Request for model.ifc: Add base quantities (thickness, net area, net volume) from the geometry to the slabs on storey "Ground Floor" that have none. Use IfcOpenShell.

First a look at what the model holds.

```python
import ifcopenshell
import ifcopenshell.util.element
import ifcopenshell.util.unit

model = ifcopenshell.open("model.ifc")
print(model.schema)
for unit_type in ("LENGTHUNIT", "AREAUNIT", "VOLUMEUNIT"):
    print(unit_type, ifcopenshell.util.unit.calculate_unit_scale(model, unit_type))
storey = next(s for s in model.by_type("IfcBuildingStorey") if s.Name == "Ground Floor")
slabs = [e for e in ifcopenshell.util.element.get_decomposition(storey) if e.is_a("IfcSlab")]
for e in sorted(slabs, key=lambda e: e.id()):
    print(e.id(), e.is_a(), e.Name, list(ifcopenshell.util.element.get_psets(e, qtos_only=True)), sep=" | ")
```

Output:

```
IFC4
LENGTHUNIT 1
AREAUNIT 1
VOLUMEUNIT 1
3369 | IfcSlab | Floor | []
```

```python
import ifcopenshell
import ifcopenshell.api.pset
import ifcopenshell.geom
import ifcopenshell.util.element
import ifcopenshell.util.shape
import ifcopenshell.util.unit

model = ifcopenshell.open("model.ifc")
unit_scale = ifcopenshell.util.unit.calculate_unit_scale(model)
area_scale = ifcopenshell.util.unit.calculate_unit_scale(model, "AREAUNIT")
volume_scale = ifcopenshell.util.unit.calculate_unit_scale(model, "VOLUMEUNIT")
settings = ifcopenshell.geom.settings()

storey = next(s for s in model.by_type("IfcBuildingStorey") if s.Name == "Ground Floor")
slabs = [e for e in ifcopenshell.util.element.get_decomposition(storey) if e.is_a("IfcSlab")]

for e in sorted(slabs, key=lambda e: e.id()):
    if ifcopenshell.util.element.get_psets(e, qtos_only=True, should_inherit=False):
        continue
    # Geometry comes back in metres, in the element's own axes.
    shape = ifcopenshell.geom.create_shape(settings, e)
    values = {
        "Width": ifcopenshell.util.shape.get_z(shape.geometry) / unit_scale,
        "NetArea": ifcopenshell.util.shape.get_footprint_area(shape.geometry) / area_scale,
        "NetVolume": ifcopenshell.util.shape.get_volume(shape.geometry) / volume_scale,
    }
    qto = ifcopenshell.api.pset.add_qto(model, product=e, name="Qto_SlabBaseQuantities")
    ifcopenshell.api.pset.edit_qto(model, qto=qto, properties=values)
    print(e.id(), {k: round(v, 3) for k, v in values.items()})

model.write("model_v2.ifc")
```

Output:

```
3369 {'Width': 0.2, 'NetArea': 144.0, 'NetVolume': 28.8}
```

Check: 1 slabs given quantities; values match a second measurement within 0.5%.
